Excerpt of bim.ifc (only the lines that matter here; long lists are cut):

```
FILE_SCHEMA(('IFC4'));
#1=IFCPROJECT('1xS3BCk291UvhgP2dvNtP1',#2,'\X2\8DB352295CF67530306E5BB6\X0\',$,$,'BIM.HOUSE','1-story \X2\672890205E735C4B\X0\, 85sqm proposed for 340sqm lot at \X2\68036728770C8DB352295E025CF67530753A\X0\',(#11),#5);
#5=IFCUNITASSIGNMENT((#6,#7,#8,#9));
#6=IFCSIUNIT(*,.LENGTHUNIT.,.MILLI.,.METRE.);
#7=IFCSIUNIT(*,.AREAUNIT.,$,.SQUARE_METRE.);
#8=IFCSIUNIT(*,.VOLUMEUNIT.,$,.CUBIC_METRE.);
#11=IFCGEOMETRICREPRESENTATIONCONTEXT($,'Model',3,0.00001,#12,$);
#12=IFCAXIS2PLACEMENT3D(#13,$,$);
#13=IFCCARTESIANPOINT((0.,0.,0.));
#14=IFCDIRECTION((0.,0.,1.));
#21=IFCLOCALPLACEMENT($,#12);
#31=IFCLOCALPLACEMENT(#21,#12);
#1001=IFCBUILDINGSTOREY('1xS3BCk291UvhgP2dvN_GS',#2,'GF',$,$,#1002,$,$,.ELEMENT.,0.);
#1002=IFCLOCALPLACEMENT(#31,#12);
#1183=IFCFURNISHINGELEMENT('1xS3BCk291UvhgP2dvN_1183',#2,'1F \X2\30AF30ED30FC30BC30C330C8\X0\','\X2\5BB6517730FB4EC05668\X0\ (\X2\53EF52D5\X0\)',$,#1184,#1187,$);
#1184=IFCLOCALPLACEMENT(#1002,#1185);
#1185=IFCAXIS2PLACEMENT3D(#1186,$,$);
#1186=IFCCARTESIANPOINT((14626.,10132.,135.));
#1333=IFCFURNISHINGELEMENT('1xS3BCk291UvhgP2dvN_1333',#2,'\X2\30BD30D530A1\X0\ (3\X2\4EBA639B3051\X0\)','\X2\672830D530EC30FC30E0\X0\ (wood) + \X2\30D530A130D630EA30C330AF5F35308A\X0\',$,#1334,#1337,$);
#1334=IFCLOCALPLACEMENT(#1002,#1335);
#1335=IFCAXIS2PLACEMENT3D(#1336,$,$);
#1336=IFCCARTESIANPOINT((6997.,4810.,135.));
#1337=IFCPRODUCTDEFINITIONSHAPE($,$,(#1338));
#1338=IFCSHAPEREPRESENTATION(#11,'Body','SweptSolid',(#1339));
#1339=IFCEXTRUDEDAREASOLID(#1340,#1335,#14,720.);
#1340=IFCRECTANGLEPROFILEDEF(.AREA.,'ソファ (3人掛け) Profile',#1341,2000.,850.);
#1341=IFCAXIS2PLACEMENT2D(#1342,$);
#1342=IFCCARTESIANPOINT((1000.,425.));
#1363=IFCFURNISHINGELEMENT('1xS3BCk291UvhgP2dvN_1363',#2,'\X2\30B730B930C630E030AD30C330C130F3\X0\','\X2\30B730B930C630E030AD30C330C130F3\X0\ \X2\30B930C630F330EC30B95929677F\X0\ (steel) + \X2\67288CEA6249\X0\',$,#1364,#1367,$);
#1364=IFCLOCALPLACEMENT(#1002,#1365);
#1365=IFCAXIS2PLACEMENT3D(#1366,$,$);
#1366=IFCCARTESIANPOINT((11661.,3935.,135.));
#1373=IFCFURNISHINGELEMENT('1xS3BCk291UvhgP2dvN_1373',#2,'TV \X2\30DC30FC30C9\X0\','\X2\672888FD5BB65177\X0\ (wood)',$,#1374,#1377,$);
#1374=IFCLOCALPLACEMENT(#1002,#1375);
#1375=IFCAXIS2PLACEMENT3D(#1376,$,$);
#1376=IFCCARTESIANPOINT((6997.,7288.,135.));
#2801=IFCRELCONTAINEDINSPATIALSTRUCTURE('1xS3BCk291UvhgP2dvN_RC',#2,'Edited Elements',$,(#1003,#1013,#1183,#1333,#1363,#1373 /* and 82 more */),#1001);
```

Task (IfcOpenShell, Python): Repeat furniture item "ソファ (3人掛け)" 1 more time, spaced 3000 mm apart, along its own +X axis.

```python
import ifcopenshell
import ifcopenshell.api.geometry
import ifcopenshell.api.root
import ifcopenshell.util.element
import ifcopenshell.util.placement
import ifcopenshell.util.unit

model = ifcopenshell.open("bim.ifc")
unit_scale = ifcopenshell.util.unit.calculate_unit_scale(model)


def reuse_history(source, copy):
    """copy_class also copies each property set's owner history, people and application; keep the originals."""
    for rel in copy.IsDefinedBy:
        if rel.is_a("IfcRelDefinesByProperties") and (history := rel.RelatingPropertyDefinition.OwnerHistory):
            rel.RelatingPropertyDefinition.OwnerHistory = source.OwnerHistory
            ifcopenshell.util.element.remove_deep2(model, history)


source = model.by_guid("1xS3BCk291UvhgP2dvN_1333")
base = ifcopenshell.util.placement.get_local_placement(source.ObjectPlacement)
step = base[:3, 0] * 3 / unit_scale

for i in range(1, 2):
    copy = ifcopenshell.api.root.copy_class(model, product=source)
    copy.Representation = ifcopenshell.util.element.copy_deep(
        model, source.Representation, exclude=["IfcGeometricRepresentationContext", "IfcRepresentationMap"]
    )
    reuse_history(source, copy)
    matrix = base.copy()
    matrix[:3, 3] += i * step
    print("added at", matrix[:3, 3].round(3) + 0.0)
    ifcopenshell.api.geometry.edit_object_placement(model, product=copy, matrix=matrix, is_si=False)

model.write("bim_edited.ifc")
```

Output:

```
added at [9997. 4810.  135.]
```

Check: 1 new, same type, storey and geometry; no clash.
